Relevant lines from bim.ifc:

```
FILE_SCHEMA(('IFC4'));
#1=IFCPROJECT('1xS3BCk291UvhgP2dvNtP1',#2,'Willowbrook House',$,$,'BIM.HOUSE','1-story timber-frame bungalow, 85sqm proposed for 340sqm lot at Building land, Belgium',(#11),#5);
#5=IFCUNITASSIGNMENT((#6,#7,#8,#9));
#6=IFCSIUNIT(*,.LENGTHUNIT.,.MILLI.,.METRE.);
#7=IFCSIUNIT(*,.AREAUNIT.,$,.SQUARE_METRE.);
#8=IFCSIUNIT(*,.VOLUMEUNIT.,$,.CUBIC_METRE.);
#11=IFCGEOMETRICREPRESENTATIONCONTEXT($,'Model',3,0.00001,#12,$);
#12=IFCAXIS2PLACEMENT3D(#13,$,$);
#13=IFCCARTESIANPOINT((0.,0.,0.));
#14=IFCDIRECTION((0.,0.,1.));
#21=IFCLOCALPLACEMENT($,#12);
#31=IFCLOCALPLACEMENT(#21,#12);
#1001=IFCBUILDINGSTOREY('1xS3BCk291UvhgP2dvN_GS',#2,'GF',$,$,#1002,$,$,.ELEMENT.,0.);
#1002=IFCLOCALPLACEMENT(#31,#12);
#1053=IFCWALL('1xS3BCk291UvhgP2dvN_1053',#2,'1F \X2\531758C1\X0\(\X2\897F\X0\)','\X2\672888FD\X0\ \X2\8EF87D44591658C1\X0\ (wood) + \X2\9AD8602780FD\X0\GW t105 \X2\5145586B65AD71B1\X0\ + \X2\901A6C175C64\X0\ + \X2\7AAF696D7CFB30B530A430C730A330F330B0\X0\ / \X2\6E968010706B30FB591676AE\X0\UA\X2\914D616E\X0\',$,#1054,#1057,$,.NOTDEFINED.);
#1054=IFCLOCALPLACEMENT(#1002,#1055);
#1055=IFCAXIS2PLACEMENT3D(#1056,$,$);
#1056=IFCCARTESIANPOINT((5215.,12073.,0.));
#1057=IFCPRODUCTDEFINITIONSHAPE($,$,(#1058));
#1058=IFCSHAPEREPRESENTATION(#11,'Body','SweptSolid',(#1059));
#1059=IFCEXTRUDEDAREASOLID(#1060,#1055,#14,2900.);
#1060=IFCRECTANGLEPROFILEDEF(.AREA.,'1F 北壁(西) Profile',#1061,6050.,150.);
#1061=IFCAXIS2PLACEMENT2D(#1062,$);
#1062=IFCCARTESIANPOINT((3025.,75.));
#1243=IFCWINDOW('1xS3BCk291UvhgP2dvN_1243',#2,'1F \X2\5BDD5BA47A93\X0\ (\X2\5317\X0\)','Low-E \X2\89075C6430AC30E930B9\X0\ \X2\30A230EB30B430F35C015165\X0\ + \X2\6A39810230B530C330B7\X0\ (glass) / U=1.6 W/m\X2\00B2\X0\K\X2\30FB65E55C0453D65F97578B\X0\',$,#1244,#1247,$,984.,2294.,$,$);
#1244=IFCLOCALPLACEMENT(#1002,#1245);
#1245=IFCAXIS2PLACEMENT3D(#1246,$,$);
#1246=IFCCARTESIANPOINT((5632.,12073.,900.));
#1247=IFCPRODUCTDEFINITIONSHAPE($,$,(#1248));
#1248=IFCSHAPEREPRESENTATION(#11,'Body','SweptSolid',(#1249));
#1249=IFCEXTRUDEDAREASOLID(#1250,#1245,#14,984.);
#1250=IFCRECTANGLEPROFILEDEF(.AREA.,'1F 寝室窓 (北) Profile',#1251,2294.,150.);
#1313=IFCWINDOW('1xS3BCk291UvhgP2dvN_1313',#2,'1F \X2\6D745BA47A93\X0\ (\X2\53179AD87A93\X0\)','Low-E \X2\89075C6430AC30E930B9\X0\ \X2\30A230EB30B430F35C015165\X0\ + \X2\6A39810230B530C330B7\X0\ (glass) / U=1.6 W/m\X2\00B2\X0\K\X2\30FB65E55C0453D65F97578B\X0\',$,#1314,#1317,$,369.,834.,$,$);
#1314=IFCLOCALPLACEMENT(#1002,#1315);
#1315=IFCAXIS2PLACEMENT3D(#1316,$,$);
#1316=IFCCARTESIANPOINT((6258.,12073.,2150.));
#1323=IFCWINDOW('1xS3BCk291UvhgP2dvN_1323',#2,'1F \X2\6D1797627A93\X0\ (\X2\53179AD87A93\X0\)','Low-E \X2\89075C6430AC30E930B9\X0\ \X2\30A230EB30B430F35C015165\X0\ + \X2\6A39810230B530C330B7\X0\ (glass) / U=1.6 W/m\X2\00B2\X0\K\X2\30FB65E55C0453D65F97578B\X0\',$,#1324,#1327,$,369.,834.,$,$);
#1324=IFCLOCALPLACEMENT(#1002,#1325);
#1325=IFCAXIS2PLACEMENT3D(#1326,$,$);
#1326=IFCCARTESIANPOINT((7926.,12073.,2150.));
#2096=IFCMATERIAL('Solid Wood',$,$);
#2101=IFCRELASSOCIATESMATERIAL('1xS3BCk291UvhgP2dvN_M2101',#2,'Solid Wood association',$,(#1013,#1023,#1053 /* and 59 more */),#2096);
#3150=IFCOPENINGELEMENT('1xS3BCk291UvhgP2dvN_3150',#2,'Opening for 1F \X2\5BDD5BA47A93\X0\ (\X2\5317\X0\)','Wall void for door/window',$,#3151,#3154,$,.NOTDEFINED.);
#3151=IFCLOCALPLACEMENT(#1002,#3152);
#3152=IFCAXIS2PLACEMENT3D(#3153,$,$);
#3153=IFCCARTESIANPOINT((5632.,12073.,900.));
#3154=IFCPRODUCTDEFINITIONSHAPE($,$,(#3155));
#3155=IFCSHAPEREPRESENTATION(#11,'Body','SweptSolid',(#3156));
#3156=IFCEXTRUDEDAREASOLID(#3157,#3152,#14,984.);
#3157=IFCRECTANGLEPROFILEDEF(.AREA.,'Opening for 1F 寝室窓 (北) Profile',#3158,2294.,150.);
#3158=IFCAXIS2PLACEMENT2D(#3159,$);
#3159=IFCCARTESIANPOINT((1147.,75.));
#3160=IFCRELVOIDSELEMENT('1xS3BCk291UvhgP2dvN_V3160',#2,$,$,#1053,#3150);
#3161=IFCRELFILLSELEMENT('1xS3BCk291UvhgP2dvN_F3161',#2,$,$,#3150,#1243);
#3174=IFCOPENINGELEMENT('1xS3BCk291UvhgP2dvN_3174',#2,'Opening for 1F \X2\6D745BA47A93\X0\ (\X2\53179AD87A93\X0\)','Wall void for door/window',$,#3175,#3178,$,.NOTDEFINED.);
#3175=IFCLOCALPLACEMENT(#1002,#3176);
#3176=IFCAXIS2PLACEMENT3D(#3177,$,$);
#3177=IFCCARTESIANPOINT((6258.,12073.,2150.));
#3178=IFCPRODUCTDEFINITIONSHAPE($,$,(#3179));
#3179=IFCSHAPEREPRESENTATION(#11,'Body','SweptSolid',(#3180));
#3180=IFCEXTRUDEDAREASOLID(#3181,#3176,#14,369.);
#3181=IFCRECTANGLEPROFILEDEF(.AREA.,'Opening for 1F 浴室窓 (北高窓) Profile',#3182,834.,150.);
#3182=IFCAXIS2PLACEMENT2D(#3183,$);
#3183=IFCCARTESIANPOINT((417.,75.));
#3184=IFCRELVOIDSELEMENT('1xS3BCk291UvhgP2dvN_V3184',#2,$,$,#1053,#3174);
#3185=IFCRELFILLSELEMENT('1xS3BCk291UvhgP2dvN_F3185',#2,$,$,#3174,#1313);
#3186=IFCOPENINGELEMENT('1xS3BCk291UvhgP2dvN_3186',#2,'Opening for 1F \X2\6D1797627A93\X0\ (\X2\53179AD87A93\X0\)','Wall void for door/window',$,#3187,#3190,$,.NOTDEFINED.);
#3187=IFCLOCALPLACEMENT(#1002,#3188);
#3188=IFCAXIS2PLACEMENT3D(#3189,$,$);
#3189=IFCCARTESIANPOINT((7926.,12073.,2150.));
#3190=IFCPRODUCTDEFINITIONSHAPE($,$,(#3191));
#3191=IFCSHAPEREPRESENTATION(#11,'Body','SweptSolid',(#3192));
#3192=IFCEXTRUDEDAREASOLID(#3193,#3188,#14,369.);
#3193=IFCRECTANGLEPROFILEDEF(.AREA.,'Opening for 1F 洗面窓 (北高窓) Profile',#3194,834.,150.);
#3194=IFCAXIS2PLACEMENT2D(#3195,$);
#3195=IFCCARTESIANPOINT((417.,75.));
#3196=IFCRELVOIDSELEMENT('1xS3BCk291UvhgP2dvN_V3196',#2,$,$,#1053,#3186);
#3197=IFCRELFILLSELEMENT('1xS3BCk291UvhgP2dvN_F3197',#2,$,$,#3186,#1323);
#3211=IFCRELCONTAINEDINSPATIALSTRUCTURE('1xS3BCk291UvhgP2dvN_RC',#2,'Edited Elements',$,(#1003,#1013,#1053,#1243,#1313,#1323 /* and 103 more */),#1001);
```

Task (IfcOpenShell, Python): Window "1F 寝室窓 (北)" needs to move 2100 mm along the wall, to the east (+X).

```python
import ifcopenshell
import ifcopenshell.api.geometry
import ifcopenshell.util.placement
import ifcopenshell.util.unit

model = ifcopenshell.open("bim.ifc")
unit_scale = ifcopenshell.util.unit.calculate_unit_scale(model)

window = model.by_guid("1xS3BCk291UvhgP2dvN_1243")
opening = window.FillsVoids[0].RelatingOpeningElement
wall = opening.VoidsElements[0].RelatingBuildingElement

wall_matrix = ifcopenshell.util.placement.get_local_placement(wall.ObjectPlacement)
shift = wall_matrix[:3, 0] * 2.1 / unit_scale
before = ifcopenshell.util.placement.get_local_placement(window.ObjectPlacement)[:3, 3].copy()

# The window is not placed relative to its opening, so move both.
for product in (opening, window):
    matrix = ifcopenshell.util.placement.get_local_placement(product.ObjectPlacement)
    matrix[:3, 3] += shift
    ifcopenshell.api.geometry.edit_object_placement(model, product=product, matrix=matrix, is_si=False)

after = ifcopenshell.util.placement.get_local_placement(window.ObjectPlacement)[:3, 3]
print("window moved by", (after - before).round(3) + 0.0)

model.write("bim-out.ifc")
```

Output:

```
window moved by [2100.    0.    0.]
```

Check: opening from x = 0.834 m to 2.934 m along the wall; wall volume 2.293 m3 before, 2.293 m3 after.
